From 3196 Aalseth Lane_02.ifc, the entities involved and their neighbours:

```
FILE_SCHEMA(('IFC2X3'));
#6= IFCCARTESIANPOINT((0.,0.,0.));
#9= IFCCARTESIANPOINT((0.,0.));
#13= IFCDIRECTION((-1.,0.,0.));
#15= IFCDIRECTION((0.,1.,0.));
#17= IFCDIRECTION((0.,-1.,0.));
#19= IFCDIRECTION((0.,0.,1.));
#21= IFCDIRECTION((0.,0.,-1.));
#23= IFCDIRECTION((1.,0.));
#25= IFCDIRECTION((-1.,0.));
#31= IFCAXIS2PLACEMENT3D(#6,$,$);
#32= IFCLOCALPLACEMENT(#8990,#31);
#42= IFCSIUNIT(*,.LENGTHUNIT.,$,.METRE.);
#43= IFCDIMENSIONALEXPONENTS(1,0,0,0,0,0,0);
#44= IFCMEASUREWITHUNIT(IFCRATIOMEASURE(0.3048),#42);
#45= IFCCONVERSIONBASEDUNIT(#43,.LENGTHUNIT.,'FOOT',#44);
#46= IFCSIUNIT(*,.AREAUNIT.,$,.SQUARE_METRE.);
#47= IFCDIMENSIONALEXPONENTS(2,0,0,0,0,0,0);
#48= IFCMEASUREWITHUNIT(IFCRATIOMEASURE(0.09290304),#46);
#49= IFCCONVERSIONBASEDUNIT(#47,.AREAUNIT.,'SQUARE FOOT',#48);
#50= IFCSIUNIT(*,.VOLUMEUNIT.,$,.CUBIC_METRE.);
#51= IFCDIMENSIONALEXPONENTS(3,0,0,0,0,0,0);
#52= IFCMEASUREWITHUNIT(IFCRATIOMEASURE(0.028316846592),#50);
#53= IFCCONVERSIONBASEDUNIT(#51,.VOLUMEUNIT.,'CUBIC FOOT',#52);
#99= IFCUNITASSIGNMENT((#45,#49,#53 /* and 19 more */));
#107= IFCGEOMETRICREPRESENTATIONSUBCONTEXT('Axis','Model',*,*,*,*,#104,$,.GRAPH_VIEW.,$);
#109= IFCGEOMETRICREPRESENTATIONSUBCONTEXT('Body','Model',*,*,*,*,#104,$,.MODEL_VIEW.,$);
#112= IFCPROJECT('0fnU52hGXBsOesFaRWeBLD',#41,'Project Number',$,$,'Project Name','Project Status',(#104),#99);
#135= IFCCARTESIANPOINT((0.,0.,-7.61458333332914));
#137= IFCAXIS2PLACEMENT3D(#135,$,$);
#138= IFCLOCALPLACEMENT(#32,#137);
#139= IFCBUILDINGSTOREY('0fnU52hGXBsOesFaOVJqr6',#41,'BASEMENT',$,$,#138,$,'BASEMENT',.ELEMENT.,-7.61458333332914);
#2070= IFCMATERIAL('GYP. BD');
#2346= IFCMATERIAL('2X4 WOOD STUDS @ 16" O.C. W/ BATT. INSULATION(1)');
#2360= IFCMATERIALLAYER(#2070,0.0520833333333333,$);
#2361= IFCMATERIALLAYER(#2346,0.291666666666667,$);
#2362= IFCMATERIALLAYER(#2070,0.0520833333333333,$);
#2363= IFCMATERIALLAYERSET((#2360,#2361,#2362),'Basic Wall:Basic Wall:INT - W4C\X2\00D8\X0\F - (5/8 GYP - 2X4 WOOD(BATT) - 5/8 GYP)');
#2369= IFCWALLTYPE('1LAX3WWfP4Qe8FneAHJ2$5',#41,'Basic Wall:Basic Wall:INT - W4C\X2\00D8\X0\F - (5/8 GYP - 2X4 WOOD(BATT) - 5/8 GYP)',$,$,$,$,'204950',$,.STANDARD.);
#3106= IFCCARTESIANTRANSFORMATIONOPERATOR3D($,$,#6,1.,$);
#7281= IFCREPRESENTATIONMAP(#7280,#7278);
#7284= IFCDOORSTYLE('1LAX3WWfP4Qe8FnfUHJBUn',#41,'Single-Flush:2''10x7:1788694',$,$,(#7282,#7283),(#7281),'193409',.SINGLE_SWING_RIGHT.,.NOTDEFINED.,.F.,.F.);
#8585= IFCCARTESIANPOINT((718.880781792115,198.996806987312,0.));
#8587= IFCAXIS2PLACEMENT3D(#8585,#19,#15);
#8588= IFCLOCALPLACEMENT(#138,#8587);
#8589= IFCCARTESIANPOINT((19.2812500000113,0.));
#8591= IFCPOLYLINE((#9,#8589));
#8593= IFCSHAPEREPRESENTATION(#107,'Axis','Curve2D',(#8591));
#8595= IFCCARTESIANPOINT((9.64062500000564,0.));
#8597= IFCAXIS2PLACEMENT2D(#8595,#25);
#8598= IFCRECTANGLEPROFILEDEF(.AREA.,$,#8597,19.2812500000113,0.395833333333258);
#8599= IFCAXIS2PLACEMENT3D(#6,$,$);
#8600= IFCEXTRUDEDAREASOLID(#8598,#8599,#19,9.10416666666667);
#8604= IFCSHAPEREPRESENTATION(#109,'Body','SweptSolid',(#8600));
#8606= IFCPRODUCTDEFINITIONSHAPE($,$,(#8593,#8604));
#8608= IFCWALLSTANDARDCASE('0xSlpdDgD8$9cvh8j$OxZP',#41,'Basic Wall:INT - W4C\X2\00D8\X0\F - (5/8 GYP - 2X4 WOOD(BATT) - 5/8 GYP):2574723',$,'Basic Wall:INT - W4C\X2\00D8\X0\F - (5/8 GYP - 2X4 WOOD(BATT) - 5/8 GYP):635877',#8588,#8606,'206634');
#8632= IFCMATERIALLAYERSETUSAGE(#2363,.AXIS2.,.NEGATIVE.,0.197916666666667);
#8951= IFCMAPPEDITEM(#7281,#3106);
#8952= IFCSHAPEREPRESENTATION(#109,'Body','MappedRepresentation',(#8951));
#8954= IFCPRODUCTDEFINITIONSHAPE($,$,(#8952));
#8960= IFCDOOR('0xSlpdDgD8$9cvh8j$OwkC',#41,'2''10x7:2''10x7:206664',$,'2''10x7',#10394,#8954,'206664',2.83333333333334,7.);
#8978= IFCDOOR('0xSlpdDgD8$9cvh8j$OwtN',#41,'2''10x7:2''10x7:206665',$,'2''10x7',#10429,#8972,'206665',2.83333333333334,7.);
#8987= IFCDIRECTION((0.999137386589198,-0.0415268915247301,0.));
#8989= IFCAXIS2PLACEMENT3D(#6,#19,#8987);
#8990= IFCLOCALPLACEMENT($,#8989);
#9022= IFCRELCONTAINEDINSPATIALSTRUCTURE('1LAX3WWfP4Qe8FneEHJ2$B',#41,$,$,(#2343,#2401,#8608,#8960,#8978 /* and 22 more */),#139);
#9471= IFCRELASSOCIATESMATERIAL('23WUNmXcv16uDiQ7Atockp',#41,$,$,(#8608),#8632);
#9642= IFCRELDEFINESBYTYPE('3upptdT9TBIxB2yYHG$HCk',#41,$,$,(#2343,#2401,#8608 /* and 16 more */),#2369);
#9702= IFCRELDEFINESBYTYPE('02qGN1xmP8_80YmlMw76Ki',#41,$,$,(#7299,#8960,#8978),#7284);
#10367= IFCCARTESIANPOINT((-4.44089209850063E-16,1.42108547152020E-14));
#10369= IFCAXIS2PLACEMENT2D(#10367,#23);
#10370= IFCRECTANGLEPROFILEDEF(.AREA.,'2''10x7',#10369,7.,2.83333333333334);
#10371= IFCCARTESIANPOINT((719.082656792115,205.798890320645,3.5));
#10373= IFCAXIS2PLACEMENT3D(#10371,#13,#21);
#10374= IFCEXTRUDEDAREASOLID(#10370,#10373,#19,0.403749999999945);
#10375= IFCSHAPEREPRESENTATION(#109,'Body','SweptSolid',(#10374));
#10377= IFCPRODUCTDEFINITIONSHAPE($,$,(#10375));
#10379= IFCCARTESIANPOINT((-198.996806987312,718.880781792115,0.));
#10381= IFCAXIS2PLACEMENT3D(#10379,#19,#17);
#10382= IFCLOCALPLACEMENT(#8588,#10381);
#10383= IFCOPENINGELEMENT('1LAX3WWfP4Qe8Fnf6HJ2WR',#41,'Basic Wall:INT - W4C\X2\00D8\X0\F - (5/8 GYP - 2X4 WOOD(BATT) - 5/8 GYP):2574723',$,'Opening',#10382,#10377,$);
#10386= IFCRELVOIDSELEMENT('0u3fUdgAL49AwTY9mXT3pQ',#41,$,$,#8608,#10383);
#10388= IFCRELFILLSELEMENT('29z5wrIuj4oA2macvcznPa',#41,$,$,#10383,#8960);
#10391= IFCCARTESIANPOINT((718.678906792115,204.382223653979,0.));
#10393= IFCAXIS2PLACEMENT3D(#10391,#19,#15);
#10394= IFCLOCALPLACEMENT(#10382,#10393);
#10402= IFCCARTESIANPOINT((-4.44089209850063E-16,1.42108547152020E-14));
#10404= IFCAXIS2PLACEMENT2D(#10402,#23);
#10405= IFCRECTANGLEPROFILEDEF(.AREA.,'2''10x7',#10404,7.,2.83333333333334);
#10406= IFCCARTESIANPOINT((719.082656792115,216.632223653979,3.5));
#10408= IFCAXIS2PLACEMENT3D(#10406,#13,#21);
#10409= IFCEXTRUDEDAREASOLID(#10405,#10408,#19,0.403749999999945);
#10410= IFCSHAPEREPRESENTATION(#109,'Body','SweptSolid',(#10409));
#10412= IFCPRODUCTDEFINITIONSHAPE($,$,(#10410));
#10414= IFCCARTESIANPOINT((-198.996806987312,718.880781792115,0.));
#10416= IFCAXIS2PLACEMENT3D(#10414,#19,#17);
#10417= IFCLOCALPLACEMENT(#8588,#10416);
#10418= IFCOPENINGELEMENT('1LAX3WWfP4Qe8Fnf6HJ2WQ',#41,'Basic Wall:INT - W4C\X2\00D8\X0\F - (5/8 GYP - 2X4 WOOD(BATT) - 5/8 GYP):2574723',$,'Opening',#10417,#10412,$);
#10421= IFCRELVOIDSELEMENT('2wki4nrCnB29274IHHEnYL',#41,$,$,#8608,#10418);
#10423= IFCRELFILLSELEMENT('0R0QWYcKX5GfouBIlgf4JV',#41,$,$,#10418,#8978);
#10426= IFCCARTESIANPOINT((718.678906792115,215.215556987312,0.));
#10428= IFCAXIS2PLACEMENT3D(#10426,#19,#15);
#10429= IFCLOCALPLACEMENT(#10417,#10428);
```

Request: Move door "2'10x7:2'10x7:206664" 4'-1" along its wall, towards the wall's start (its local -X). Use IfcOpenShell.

```python
import ifcopenshell
import ifcopenshell.api.geometry
import ifcopenshell.util.placement
import ifcopenshell.util.unit

model = ifcopenshell.open("3196 Aalseth Lane_02.ifc")
unit_scale = ifcopenshell.util.unit.calculate_unit_scale(model)

door = model.by_guid("0xSlpdDgD8$9cvh8j$OwkC")
opening = door.FillsVoids[0].RelatingOpeningElement
wall = opening.VoidsElements[0].RelatingBuildingElement

wall_matrix = ifcopenshell.util.placement.get_local_placement(wall.ObjectPlacement)
shift = wall_matrix[:3, 0] * -49 * 0.0254 / unit_scale
before = ifcopenshell.util.placement.get_local_placement(door.ObjectPlacement)[:3, 3].copy()

# The door is placed relative to its opening, so it follows when the opening moves.
matrix = ifcopenshell.util.placement.get_local_placement(opening.ObjectPlacement)
matrix[:3, 3] += shift
ifcopenshell.api.geometry.edit_object_placement(
    model, product=opening, matrix=matrix, is_si=False, should_transform_children=True
)

after = ifcopenshell.util.placement.get_local_placement(door.ObjectPlacement)[:3, 3]
print("door moved by", (after - before).round(3) + 0.0)

model.write("3196 Aalseth Lane_02-out.ifc")
```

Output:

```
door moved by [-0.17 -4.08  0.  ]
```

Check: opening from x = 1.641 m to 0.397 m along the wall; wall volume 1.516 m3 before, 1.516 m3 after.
